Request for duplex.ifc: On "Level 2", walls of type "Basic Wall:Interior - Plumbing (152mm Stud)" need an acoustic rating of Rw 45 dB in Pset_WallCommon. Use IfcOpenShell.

First a look at what the model holds.

```python
import ifcopenshell
import ifcopenshell.util.element

model = ifcopenshell.open("duplex.ifc")
print(model.schema)
storey = next(s for s in model.by_type("IfcBuildingStorey") if s.Name == "Level 2")
walls = [e for e in ifcopenshell.util.element.get_decomposition(storey) if e.is_a("IfcWall")]
seen = {}
for e in walls:
    element_type = ifcopenshell.util.element.get_type(e)
    key = (element_type.Name if element_type != e and element_type else None, ifcopenshell.util.element.get_pset(e, "Pset_WallCommon", "AcousticRating"))
    seen[key] = seen.get(key, 0) + 1
for (name, value), count in sorted(seen.items(), key=str):
    print(count, "x", name, "|", value)
```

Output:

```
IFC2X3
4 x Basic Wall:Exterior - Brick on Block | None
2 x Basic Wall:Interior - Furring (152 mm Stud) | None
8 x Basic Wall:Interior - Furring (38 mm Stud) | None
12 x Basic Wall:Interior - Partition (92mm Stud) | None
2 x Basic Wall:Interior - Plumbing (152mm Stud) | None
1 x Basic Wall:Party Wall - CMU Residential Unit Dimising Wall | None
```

```python
import ifcopenshell
import ifcopenshell.api.pset
import ifcopenshell.util.element

model = ifcopenshell.open("duplex.ifc")

storey = next(s for s in model.by_type("IfcBuildingStorey") if s.Name == "Level 2")
walls = [e for e in ifcopenshell.util.element.get_decomposition(storey) if e.is_a("IfcWall")]

count = 0
for e in walls:
    element_type = ifcopenshell.util.element.get_type(e)
    if element_type in (None, e) or element_type.Name != "Basic Wall:Interior - Plumbing (152mm Stud)":
        continue
    # add_pset returns the element's existing set when there is one.
    pset = ifcopenshell.api.pset.add_pset(model, product=e, name="Pset_WallCommon")
    ifcopenshell.api.pset.edit_pset(model, pset=pset, properties={"AcousticRating": "Rw 45 dB"})
    count += 1

print(count, "walls updated")

model.write("duplex_updated.ifc")
```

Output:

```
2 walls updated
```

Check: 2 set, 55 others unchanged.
